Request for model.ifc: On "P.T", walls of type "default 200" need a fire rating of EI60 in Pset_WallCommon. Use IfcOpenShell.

First a look at what the model holds.

```python
import ifcopenshell
import ifcopenshell.util.element

model = ifcopenshell.open("model.ifc")
print(model.schema)
storey = next(s for s in model.by_type("IfcBuildingStorey") if s.Name == "P.T")
walls = [e for e in ifcopenshell.util.element.get_decomposition(storey) if e.is_a("IfcWall")]
seen = {}
for e in walls:
    element_type = ifcopenshell.util.element.get_type(e)
    key = (element_type.Name if element_type != e and element_type else None, ifcopenshell.util.element.get_pset(e, "Pset_WallCommon", "FireRating"))
    seen[key] = seen.get(key, 0) + 1
for (name, value), count in sorted(seen.items(), key=str):
    print(count, "x", name, "|", value)
```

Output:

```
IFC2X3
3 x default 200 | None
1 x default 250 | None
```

```python
import ifcopenshell
import ifcopenshell.api.pset
import ifcopenshell.util.element

model = ifcopenshell.open("model.ifc")

storey = next(s for s in model.by_type("IfcBuildingStorey") if s.Name == "P.T")
walls = [e for e in ifcopenshell.util.element.get_decomposition(storey) if e.is_a("IfcWall")]

count = 0
for e in walls:
    element_type = ifcopenshell.util.element.get_type(e)
    if element_type in (None, e) or element_type.Name != "default 200":
        continue
    # add_pset returns the element's existing set when there is one.
    pset = ifcopenshell.api.pset.add_pset(model, product=e, name="Pset_WallCommon")
    ifcopenshell.api.pset.edit_pset(model, pset=pset, properties={"FireRating": "EI60"})
    count += 1

print(count, "walls updated")

model.write("model_updated.ifc")
```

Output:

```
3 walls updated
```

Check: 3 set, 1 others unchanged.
